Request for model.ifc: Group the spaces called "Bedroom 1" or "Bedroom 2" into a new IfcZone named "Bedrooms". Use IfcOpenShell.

First a look at what the model holds.

```python
import ifcopenshell

model = ifcopenshell.open("model.ifc")
print(model.schema)
seen = {}
for space in model.by_type("IfcSpace"):
    seen[space.LongName] = seen.get(space.LongName, 0) + 1
for name, count in sorted(seen.items(), key=str):
    print(count, "x", name)
print("zones:", [z.Name for z in model.by_type("IfcZone")][:20])
```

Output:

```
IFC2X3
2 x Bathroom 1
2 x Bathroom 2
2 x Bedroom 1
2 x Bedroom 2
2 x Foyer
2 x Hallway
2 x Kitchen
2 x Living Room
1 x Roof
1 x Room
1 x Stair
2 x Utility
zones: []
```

```python
import ifcopenshell
import ifcopenshell.api.group
import ifcopenshell.api.root

model = ifcopenshell.open("model.ifc")

names = {"Bedroom 1", "Bedroom 2"}
spaces = [s for s in model.by_type("IfcSpace") if s.LongName in names]

zone = ifcopenshell.api.root.create_entity(model, ifc_class="IfcZone", name="Bedrooms")
ifcopenshell.api.group.assign_group(model, products=spaces, group=zone)
print(len(spaces), "spaces in", zone.Name)

model.write("model_updated.ifc")
```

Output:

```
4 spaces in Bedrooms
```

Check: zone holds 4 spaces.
